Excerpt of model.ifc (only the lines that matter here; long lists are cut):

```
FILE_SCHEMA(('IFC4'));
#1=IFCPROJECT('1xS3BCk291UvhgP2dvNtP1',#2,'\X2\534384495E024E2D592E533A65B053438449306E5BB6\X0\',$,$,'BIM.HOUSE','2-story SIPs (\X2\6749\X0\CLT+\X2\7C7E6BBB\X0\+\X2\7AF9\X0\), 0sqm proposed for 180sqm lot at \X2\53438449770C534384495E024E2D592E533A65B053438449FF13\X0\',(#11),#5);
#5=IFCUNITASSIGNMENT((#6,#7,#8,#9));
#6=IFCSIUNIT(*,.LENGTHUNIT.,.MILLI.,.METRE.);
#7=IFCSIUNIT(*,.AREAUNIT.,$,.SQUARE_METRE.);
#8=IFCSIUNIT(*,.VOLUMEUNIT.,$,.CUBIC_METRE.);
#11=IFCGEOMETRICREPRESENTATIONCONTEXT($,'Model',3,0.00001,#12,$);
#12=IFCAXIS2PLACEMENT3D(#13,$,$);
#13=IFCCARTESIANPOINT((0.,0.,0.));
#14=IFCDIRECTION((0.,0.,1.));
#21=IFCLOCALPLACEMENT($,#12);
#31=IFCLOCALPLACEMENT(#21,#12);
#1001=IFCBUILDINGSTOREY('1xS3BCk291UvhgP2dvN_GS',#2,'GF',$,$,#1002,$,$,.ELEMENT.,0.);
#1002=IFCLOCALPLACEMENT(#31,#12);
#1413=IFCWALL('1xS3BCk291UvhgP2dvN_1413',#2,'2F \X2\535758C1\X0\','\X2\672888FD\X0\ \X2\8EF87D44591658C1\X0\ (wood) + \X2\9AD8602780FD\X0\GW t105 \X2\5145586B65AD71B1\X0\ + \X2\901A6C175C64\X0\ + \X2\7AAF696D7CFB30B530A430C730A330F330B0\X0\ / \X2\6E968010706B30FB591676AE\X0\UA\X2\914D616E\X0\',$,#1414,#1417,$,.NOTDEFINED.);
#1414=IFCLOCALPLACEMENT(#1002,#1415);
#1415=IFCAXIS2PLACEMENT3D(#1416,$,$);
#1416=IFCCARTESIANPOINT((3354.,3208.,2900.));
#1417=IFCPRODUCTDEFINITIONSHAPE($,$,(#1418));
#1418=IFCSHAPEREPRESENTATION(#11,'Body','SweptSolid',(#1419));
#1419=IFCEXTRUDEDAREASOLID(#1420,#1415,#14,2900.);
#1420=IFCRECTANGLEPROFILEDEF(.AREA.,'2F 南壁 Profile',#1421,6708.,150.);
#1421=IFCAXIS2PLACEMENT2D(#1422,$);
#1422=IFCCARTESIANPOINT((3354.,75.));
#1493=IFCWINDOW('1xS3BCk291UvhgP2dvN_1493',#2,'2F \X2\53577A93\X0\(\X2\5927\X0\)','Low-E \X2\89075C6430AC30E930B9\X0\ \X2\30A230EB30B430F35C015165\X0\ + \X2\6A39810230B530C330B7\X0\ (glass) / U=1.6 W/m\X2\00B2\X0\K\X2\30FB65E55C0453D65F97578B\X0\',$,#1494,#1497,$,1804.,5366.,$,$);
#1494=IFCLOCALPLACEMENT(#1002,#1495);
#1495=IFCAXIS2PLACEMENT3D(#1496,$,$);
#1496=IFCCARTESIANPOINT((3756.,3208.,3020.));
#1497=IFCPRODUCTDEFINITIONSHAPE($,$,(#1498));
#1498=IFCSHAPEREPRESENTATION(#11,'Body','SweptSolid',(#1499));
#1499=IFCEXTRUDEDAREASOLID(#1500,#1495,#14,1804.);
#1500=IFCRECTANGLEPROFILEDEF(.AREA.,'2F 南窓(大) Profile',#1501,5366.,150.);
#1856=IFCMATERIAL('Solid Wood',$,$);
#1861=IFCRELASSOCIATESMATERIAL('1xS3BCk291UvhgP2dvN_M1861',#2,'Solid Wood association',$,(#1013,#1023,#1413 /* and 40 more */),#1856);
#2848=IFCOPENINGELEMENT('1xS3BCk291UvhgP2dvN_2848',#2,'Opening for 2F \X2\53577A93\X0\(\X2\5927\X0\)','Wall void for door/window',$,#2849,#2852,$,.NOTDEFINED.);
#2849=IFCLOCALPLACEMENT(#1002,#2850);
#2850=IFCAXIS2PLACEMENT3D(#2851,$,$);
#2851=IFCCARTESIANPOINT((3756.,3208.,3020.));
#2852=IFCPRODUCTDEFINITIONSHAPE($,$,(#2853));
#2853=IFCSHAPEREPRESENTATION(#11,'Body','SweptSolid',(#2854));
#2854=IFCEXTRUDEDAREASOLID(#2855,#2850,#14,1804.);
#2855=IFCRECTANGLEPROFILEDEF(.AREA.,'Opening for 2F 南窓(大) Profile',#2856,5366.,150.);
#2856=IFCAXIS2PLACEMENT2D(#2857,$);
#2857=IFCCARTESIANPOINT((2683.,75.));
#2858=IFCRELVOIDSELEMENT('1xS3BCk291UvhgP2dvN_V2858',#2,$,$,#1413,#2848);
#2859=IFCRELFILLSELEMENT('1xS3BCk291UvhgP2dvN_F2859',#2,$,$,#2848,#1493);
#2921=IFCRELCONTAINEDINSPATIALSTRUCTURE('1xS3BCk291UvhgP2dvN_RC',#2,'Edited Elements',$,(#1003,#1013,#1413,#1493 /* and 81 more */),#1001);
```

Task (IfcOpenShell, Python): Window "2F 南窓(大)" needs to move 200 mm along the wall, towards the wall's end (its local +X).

```python
import ifcopenshell
import ifcopenshell.api.geometry
import ifcopenshell.util.placement
import ifcopenshell.util.unit

model = ifcopenshell.open("model.ifc")
unit_scale = ifcopenshell.util.unit.calculate_unit_scale(model)

window = model.by_id(1493)
opening = window.FillsVoids[0].RelatingOpeningElement
wall = opening.VoidsElements[0].RelatingBuildingElement

wall_matrix = ifcopenshell.util.placement.get_local_placement(wall.ObjectPlacement)
shift = wall_matrix[:3, 0] * 0.2 / unit_scale
before = ifcopenshell.util.placement.get_local_placement(window.ObjectPlacement)[:3, 3].copy()

# The window is not placed relative to its opening, so move both.
for product in (opening, window):
    matrix = ifcopenshell.util.placement.get_local_placement(product.ObjectPlacement)
    matrix[:3, 3] += shift
    ifcopenshell.api.geometry.edit_object_placement(model, product=product, matrix=matrix, is_si=False)

after = ifcopenshell.util.placement.get_local_placement(window.ObjectPlacement)[:3, 3]
print("window moved by", (after - before).round(3) + 0.0)

model.write("model-out.ifc")
```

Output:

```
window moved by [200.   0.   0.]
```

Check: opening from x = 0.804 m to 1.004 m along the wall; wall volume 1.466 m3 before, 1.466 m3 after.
